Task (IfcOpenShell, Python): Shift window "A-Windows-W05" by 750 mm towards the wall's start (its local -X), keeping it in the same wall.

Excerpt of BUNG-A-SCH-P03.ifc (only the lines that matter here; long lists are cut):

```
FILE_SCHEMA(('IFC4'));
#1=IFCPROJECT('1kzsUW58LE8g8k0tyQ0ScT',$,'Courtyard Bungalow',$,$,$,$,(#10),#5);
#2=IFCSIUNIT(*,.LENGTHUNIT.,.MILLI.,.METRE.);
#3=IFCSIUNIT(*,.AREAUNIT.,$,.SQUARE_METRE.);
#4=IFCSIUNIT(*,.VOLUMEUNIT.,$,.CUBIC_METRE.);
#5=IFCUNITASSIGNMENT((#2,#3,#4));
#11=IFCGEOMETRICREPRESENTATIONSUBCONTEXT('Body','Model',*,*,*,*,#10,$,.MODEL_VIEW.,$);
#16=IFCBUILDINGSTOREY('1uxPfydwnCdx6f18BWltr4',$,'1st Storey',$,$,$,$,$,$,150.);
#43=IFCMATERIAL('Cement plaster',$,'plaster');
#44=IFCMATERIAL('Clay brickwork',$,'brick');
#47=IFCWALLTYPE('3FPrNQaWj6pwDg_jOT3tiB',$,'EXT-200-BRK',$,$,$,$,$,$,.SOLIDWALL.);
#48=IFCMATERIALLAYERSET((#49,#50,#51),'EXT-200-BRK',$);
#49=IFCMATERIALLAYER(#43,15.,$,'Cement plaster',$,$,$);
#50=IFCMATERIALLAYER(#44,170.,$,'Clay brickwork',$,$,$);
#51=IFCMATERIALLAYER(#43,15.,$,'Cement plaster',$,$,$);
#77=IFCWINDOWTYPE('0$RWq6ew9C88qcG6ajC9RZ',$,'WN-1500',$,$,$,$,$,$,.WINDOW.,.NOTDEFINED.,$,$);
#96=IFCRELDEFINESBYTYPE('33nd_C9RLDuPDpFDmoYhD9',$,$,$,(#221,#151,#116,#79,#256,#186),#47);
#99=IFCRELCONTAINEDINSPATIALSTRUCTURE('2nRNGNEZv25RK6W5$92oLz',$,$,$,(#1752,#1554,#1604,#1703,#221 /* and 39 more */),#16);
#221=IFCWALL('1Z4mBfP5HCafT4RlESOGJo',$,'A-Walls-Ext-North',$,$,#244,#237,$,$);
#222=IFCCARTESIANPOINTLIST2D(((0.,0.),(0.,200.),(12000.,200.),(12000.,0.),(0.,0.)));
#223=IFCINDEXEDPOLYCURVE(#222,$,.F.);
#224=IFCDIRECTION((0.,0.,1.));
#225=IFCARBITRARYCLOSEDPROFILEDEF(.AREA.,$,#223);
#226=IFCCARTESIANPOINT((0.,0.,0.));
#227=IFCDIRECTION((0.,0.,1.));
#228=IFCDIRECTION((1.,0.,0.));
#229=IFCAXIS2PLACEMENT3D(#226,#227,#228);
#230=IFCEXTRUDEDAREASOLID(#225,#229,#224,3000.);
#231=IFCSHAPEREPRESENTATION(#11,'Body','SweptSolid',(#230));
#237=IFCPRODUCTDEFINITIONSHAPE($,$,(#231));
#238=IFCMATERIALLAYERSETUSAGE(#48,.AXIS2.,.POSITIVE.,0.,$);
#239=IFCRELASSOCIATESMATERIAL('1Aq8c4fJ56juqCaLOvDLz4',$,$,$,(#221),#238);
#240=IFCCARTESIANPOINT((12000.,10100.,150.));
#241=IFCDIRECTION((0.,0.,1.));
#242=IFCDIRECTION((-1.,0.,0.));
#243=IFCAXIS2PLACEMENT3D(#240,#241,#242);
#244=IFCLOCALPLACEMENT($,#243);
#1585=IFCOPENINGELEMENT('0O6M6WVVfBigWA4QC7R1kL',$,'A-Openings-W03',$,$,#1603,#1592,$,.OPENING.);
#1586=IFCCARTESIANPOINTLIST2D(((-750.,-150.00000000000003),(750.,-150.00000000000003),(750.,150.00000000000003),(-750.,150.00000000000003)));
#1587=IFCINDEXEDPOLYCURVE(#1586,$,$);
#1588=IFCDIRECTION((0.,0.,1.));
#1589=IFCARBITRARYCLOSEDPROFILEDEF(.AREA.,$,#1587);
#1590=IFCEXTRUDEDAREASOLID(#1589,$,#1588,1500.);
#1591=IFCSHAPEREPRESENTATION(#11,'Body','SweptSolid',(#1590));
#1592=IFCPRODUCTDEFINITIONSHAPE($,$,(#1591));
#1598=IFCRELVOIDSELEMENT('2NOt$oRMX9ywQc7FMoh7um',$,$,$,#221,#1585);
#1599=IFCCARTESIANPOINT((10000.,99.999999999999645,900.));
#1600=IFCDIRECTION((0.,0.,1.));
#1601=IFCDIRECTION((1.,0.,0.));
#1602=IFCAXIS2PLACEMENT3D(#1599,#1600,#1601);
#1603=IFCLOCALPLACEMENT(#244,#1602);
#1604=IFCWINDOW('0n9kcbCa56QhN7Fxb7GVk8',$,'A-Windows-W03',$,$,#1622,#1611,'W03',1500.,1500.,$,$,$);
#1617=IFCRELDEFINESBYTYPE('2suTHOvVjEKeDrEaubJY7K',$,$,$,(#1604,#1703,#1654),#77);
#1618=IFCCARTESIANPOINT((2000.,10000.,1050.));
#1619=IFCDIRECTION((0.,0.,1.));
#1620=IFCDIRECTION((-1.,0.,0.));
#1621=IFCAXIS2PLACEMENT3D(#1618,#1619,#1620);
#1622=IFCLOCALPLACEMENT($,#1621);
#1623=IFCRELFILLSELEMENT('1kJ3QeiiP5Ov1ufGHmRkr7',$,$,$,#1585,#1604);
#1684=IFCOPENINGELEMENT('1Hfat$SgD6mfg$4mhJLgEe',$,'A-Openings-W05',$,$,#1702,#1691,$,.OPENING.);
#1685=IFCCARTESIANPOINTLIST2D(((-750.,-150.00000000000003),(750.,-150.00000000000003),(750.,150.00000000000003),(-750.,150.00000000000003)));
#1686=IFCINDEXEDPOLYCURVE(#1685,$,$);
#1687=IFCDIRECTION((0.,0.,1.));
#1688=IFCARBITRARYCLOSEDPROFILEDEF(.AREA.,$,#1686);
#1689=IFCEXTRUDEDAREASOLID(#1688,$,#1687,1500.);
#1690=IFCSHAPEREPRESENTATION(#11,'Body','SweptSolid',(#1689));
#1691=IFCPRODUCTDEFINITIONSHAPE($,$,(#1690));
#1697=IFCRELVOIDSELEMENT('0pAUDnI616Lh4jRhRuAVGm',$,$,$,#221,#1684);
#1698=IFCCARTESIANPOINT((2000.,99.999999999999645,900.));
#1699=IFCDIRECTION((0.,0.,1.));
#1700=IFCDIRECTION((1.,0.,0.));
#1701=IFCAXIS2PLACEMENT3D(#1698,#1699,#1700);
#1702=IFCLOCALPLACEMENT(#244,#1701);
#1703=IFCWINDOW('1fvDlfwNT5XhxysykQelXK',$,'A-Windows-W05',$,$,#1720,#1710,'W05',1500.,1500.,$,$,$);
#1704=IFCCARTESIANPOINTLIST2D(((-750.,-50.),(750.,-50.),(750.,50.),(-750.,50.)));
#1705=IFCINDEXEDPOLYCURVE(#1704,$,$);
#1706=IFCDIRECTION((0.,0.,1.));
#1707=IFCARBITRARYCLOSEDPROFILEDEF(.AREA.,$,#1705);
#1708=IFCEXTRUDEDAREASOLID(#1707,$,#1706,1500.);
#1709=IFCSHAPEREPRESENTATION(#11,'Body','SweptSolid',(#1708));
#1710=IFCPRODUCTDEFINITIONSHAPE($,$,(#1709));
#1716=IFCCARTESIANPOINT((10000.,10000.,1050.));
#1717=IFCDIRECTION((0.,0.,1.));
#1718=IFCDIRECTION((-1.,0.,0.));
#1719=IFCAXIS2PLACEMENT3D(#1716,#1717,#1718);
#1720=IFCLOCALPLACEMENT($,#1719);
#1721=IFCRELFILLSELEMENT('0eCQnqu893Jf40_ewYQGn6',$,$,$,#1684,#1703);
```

```python
import ifcopenshell
import ifcopenshell.api.geometry
import ifcopenshell.util.placement
import ifcopenshell.util.unit

model = ifcopenshell.open("BUNG-A-SCH-P03.ifc")
unit_scale = ifcopenshell.util.unit.calculate_unit_scale(model)

window = model.by_guid("1fvDlfwNT5XhxysykQelXK")
opening = window.FillsVoids[0].RelatingOpeningElement
wall = opening.VoidsElements[0].RelatingBuildingElement

wall_matrix = ifcopenshell.util.placement.get_local_placement(wall.ObjectPlacement)
shift = wall_matrix[:3, 0] * -0.75 / unit_scale
before = ifcopenshell.util.placement.get_local_placement(window.ObjectPlacement)[:3, 3].copy()

# The window is not placed relative to its opening, so move both.
for product in (opening, window):
    matrix = ifcopenshell.util.placement.get_local_placement(product.ObjectPlacement)
    matrix[:3, 3] += shift
    ifcopenshell.api.geometry.edit_object_placement(model, product=product, matrix=matrix, is_si=False)

after = ifcopenshell.util.placement.get_local_placement(window.ObjectPlacement)[:3, 3]
print("window moved by", (after - before).round(3) + 0.0)

model.write("BUNG-A-SCH-P03_rev.ifc")
```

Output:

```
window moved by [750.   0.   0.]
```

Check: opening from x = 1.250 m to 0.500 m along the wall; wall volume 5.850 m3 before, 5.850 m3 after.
